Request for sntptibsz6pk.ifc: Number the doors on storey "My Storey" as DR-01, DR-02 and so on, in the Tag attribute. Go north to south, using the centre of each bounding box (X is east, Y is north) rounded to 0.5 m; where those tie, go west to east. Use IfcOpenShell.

First a look at what the model holds.

```python
import ifcopenshell
import ifcopenshell.util.element
import ifcopenshell.util.placement

model = ifcopenshell.open("sntptibsz6pk.ifc")
print(model.schema)
storey = next(s for s in model.by_type("IfcBuildingStorey") if s.Name == "My Storey")
doors = [e for e in ifcopenshell.util.element.get_decomposition(storey) if e.is_a("IfcDoor")]
for e in sorted(doors, key=lambda e: e.id()):
    origin = ifcopenshell.util.placement.get_local_placement(e.ObjectPlacement)[:3, 3]
    print(e.id(), e.Tag, e.Name, origin.round(2) + 0.0, sep=" | ")
```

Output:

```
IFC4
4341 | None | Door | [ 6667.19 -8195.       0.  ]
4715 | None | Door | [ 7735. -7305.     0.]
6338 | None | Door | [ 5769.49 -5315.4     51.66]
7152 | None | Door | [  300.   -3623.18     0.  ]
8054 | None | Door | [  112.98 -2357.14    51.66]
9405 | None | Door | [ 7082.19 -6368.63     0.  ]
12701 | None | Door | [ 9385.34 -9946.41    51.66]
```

```python
import ifcopenshell
import ifcopenshell.geom
import ifcopenshell.util.element
import ifcopenshell.util.shape

model = ifcopenshell.open("sntptibsz6pk.ifc")
settings = ifcopenshell.geom.settings()
settings.set("use-world-coords", True)


def centre(element):
    shape = ifcopenshell.geom.create_shape(settings, element)
    return ifcopenshell.util.shape.get_bbox_centroid(shape.geometry)


storey = next(s for s in model.by_type("IfcBuildingStorey") if s.Name == "My Storey")
doors = [e for e in ifcopenshell.util.element.get_decomposition(storey) if e.is_a("IfcDoor")]

# Insertion points can sit at a corner or the storey origin, so sort by the geometry (in metres).
centres = {e: centre(e) for e in doors}
doors.sort(key=lambda e: (-round(centres[e][1] / 0.5), centres[e][0]))

for i, e in enumerate(doors, start=1):
    number = f"DR-{i:02d}"
    e.Tag = number
    print(e.id(), number)

model.write("sntptibsz6pk_v2.ifc")
```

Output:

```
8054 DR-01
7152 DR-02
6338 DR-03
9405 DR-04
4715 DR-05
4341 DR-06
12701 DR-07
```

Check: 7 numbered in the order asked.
